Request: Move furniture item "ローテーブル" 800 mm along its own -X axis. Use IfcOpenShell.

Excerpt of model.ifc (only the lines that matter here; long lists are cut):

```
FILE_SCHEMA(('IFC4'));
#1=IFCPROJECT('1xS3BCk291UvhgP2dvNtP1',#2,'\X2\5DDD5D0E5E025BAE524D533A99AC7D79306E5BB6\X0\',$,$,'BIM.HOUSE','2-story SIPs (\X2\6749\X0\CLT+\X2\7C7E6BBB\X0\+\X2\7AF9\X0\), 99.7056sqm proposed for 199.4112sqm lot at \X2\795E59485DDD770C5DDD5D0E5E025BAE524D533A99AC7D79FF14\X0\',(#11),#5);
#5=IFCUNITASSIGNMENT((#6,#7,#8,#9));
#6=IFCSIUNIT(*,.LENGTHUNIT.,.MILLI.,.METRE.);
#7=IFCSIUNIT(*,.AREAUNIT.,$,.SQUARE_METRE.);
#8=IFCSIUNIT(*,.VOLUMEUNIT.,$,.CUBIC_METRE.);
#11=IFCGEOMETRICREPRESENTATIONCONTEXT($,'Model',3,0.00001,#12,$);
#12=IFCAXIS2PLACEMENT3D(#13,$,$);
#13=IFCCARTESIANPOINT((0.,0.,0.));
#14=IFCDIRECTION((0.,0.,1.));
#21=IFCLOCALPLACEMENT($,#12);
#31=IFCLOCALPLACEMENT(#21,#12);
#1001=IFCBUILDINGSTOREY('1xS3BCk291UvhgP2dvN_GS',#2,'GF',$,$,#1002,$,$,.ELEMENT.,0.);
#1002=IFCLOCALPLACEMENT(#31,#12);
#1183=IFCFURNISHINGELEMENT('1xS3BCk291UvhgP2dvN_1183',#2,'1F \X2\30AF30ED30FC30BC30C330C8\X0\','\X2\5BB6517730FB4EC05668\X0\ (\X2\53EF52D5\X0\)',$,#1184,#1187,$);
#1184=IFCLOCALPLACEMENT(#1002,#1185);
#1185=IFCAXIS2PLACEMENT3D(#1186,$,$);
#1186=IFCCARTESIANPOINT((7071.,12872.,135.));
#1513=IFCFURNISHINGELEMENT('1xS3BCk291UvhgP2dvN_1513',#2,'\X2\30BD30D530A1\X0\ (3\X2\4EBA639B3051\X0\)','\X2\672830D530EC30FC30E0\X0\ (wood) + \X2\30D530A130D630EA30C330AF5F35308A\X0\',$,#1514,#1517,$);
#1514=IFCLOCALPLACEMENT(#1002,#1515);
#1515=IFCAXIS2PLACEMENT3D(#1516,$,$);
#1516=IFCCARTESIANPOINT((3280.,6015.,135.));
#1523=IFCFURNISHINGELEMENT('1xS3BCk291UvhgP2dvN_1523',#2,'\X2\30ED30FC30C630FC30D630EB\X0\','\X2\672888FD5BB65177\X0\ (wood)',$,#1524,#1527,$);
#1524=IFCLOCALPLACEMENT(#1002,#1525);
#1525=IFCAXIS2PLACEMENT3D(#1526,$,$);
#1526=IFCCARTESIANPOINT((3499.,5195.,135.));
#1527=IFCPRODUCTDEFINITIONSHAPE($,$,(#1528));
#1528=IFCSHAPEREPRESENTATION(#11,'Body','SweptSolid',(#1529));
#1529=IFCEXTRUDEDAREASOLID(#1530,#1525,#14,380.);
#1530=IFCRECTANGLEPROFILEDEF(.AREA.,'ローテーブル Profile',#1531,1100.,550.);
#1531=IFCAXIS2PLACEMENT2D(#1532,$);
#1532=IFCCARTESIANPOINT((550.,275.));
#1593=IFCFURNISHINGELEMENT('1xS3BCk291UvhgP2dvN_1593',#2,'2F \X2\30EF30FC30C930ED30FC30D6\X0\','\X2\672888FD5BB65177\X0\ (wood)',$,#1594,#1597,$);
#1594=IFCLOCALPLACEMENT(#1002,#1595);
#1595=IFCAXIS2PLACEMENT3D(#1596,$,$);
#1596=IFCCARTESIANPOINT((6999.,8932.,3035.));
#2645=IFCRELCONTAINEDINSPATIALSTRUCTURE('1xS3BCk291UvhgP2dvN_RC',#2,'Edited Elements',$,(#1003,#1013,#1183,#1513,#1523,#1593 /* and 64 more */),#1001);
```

```python
import ifcopenshell
import ifcopenshell.api.geometry
import ifcopenshell.util.placement

model = ifcopenshell.open("model.ifc")

item = model.by_id(1523)
matrix = ifcopenshell.util.placement.get_local_placement(item.ObjectPlacement)
matrix[:3, 3] -= matrix[:3, 0] * 800.0
ifcopenshell.api.geometry.edit_object_placement(model, product=item, matrix=matrix, is_si=False)

print(ifcopenshell.util.placement.get_local_placement(item.ObjectPlacement).round(3) + 0.0)

model.write("model_rev.ifc")
```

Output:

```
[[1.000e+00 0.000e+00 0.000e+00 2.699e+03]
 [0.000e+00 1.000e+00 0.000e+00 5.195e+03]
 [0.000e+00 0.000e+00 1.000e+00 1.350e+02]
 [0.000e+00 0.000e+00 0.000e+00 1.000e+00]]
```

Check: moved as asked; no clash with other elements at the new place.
